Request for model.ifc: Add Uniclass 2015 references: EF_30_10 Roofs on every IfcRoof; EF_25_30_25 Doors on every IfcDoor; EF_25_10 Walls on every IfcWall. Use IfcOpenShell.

First a look at what the model holds.

```python
import ifcopenshell

model = ifcopenshell.open("model.ifc")
print(model.schema)
print("classifications:", [c.Name for c in model.by_type("IfcClassification")])
for ifc_class in ("IfcDoor", "IfcRoof", "IfcStair", "IfcWall", "IfcWindow"):
    print(ifc_class, len(model.by_type(ifc_class)))
```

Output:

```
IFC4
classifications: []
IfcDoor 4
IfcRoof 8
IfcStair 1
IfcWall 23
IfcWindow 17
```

```python
import ifcopenshell
import ifcopenshell.api.classification

model = ifcopenshell.open("model.ifc")

system = ifcopenshell.api.classification.add_classification(model, classification="Uniclass 2015")

codes = {
    "IfcRoof": ("EF_30_10", "Roofs"),
    "IfcDoor": ("EF_25_30_25", "Doors"),
    "IfcWall": ("EF_25_10", "Walls"),
}
for ifc_class, (code, name) in codes.items():
    products = model.by_type(ifc_class)
    ifcopenshell.api.classification.add_reference(
        model, products=products, classification=system, identification=code, name=name
    )
    print(code, len(products))

model.write("model_edited.ifc")
```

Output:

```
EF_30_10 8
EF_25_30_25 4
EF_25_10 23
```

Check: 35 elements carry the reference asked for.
